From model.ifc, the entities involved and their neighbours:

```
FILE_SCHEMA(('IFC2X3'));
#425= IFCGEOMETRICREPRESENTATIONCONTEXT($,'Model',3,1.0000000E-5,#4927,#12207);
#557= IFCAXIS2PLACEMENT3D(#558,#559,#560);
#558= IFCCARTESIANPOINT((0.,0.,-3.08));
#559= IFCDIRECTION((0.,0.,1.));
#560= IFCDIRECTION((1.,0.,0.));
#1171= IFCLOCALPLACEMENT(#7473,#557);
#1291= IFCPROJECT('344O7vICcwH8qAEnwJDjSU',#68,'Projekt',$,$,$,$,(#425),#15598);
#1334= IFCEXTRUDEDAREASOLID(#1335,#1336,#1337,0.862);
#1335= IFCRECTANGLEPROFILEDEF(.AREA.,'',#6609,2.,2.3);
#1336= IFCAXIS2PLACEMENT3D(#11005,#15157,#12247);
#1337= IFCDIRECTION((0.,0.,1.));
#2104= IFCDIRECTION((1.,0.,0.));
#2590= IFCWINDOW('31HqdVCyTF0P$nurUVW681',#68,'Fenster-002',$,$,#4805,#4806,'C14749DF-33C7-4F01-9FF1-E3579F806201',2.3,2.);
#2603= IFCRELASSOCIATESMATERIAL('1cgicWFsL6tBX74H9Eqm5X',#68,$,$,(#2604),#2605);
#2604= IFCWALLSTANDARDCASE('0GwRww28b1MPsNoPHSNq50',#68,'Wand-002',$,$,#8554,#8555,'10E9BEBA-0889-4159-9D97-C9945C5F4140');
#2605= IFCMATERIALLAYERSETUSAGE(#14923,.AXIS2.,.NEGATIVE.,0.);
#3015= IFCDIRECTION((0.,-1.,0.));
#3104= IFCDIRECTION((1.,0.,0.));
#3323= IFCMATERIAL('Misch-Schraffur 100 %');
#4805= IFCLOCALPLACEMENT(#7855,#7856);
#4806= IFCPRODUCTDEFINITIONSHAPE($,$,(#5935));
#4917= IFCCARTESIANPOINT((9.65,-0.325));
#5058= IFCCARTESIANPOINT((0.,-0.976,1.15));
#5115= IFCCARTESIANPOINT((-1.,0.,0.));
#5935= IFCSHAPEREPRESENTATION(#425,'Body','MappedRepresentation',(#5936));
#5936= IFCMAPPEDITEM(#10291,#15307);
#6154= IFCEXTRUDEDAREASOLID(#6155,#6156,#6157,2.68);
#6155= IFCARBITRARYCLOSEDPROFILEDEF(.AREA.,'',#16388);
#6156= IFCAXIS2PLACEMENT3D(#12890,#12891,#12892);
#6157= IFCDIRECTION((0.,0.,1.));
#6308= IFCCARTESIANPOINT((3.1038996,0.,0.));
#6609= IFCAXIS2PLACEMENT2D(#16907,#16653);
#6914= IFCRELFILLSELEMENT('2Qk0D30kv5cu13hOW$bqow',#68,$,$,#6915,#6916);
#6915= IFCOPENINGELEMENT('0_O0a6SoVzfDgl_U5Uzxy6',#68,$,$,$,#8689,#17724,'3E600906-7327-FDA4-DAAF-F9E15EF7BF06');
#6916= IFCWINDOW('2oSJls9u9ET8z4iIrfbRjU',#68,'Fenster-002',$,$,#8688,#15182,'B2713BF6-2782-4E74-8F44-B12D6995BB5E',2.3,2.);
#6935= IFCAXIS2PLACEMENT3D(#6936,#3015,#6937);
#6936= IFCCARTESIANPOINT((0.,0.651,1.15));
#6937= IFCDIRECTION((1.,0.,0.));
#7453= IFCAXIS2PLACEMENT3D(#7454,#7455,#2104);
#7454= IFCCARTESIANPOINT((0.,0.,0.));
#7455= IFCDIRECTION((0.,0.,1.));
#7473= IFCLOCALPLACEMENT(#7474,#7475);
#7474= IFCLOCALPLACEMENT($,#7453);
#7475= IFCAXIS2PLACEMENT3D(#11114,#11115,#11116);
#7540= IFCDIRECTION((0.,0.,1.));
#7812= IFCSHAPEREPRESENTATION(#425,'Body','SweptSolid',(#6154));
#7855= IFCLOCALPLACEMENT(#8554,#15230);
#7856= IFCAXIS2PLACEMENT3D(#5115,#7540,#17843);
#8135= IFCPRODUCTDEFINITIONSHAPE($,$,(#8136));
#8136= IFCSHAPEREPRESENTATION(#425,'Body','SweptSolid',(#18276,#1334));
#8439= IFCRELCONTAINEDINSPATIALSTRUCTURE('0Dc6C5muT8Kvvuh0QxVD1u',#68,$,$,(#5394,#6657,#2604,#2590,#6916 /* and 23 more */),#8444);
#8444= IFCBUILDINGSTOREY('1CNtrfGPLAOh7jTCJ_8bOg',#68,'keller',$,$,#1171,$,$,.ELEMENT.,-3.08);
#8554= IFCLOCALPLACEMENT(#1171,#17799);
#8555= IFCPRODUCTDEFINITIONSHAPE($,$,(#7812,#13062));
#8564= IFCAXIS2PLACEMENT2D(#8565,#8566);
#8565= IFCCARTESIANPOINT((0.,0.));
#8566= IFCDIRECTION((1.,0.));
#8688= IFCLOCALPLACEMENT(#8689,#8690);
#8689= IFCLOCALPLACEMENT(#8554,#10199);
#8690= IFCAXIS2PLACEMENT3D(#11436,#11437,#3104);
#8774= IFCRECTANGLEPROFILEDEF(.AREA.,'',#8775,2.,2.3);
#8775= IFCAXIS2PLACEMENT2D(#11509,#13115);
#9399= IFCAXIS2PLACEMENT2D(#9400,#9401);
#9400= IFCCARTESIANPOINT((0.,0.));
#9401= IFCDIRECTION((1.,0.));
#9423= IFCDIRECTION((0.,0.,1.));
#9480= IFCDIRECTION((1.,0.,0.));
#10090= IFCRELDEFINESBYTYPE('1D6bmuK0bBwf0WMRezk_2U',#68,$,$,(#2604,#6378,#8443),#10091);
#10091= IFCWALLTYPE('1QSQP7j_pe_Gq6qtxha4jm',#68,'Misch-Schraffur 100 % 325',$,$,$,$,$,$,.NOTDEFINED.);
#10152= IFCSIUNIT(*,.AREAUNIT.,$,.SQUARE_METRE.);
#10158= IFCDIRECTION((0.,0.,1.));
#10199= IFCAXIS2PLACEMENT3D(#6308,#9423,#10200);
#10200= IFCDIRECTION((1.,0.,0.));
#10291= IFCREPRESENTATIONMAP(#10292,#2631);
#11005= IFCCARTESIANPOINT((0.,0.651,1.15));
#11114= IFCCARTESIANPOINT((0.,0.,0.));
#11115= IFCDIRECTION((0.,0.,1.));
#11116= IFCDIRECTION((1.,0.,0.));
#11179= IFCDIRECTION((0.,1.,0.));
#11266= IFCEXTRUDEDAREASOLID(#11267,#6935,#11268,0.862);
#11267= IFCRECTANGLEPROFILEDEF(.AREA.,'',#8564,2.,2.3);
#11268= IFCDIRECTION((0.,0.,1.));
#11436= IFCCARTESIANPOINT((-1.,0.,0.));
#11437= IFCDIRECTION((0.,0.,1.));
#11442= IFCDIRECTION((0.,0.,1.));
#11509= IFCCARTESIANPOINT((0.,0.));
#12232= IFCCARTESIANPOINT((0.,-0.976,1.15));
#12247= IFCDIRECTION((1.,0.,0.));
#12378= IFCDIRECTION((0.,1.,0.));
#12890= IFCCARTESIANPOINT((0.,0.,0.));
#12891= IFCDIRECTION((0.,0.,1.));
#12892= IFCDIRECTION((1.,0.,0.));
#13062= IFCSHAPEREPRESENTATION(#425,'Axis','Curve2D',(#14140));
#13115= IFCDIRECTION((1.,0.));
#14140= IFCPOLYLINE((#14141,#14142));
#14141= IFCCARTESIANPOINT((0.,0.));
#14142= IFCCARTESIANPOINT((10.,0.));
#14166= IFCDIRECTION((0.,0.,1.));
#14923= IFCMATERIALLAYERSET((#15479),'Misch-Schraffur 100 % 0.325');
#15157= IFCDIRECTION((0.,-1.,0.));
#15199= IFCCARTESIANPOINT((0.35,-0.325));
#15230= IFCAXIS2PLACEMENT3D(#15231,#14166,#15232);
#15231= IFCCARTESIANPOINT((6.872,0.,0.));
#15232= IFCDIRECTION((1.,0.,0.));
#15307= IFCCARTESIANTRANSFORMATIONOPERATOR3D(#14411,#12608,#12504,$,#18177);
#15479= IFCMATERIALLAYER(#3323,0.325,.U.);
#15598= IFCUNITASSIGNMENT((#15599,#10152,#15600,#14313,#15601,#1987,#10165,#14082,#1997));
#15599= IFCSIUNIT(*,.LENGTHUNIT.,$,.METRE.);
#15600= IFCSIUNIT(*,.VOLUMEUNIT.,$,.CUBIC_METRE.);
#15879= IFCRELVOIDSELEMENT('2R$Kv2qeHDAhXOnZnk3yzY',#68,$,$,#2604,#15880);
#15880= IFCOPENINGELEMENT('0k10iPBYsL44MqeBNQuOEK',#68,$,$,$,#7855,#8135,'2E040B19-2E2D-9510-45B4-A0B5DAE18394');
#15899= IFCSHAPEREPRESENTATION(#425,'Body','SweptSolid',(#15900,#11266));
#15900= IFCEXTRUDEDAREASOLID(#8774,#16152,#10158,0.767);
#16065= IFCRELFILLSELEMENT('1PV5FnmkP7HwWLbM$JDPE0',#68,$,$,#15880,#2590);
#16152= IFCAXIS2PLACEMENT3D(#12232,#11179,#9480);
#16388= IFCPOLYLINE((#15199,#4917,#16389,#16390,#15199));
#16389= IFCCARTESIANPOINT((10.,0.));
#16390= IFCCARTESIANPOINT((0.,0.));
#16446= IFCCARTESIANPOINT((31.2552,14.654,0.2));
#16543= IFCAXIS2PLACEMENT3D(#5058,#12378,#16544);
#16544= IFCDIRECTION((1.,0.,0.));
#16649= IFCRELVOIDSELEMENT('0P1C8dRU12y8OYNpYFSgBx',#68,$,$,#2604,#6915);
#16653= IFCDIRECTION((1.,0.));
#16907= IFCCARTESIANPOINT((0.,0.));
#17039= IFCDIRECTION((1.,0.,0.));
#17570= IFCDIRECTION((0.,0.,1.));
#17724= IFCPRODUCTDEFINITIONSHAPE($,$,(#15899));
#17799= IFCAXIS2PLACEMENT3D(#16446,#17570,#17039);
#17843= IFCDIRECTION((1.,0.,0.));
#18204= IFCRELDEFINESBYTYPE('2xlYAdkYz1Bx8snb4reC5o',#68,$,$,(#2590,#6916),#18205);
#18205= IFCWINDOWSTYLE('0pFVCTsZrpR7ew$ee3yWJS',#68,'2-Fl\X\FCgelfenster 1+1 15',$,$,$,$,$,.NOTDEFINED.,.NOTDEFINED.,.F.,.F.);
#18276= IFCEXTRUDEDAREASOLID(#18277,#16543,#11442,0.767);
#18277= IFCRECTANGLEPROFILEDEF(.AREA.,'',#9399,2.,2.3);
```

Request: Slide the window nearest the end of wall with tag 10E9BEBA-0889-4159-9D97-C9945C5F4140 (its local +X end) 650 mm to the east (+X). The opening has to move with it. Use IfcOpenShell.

```python
import ifcopenshell
import ifcopenshell.api.geometry
import ifcopenshell.util.placement
import ifcopenshell.util.unit

model = ifcopenshell.open("model.ifc")
unit_scale = ifcopenshell.util.unit.calculate_unit_scale(model)

window = model.by_id(2590)
opening = window.FillsVoids[0].RelatingOpeningElement
wall = opening.VoidsElements[0].RelatingBuildingElement

wall_matrix = ifcopenshell.util.placement.get_local_placement(wall.ObjectPlacement)
shift = wall_matrix[:3, 0] * 0.65 / unit_scale
before = ifcopenshell.util.placement.get_local_placement(window.ObjectPlacement)[:3, 3].copy()

# The window is placed relative to its opening, so it follows when the opening moves.
matrix = ifcopenshell.util.placement.get_local_placement(opening.ObjectPlacement)
matrix[:3, 3] += shift
ifcopenshell.api.geometry.edit_object_placement(
    model, product=opening, matrix=matrix, is_si=False, should_transform_children=True
)

after = ifcopenshell.util.placement.get_local_placement(window.ObjectPlacement)[:3, 3]
print("window moved by", (after - before).round(3) + 0.0)

model.write("model-out.ifc")
```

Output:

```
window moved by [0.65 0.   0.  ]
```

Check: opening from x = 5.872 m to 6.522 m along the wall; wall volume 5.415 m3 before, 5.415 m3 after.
